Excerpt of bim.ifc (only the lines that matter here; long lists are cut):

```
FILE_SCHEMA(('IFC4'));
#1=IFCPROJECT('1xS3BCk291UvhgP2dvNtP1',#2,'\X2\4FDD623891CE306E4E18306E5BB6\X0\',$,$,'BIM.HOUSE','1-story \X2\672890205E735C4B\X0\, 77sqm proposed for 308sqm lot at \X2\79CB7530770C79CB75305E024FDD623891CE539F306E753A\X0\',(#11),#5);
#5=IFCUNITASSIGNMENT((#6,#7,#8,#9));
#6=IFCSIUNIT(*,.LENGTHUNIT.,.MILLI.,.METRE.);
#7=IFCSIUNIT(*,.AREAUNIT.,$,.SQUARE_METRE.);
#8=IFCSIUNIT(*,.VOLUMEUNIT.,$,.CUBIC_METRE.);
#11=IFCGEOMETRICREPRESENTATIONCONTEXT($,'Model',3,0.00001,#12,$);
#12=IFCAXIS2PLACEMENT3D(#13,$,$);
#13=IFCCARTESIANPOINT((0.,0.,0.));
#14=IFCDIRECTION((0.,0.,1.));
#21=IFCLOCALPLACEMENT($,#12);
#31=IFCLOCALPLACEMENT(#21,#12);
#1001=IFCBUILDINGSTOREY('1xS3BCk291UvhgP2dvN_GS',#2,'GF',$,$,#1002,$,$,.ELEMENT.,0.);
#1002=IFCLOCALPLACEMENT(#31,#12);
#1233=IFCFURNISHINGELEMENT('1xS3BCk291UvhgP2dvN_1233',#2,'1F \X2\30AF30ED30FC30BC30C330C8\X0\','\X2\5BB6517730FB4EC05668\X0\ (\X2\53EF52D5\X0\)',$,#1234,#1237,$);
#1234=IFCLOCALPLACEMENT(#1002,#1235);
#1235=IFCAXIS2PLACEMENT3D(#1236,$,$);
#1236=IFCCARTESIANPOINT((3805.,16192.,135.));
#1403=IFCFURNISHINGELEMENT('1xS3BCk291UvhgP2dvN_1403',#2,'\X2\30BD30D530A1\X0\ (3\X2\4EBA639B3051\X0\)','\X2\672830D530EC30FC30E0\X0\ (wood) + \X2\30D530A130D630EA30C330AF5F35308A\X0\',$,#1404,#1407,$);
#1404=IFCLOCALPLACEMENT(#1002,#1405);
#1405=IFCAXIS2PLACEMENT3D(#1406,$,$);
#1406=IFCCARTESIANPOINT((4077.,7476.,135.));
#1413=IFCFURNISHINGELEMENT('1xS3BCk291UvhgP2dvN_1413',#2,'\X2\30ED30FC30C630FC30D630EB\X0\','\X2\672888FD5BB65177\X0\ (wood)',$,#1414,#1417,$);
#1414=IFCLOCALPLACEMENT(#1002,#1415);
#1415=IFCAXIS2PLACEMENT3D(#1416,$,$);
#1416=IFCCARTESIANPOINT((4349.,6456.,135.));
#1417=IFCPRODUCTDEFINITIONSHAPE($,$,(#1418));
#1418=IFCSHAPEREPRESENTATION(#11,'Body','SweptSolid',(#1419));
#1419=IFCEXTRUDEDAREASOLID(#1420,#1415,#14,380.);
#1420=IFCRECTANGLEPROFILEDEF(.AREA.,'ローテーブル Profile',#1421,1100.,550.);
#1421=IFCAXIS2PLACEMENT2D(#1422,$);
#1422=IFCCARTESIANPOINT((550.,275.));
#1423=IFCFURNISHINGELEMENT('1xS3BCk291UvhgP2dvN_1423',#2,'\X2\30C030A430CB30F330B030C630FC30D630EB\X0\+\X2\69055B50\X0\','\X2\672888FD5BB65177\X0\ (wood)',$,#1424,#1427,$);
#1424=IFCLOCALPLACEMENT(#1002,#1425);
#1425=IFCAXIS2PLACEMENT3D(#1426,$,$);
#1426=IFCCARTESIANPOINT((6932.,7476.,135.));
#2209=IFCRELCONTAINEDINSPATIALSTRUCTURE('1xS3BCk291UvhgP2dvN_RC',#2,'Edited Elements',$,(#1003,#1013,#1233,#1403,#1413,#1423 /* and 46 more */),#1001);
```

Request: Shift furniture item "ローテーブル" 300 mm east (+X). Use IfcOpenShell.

```python
import ifcopenshell
import ifcopenshell.api.geometry
import ifcopenshell.util.placement

model = ifcopenshell.open("bim.ifc")

item = model.by_id(1413)
matrix = ifcopenshell.util.placement.get_local_placement(item.ObjectPlacement)
matrix[0, 3] += 300.0
ifcopenshell.api.geometry.edit_object_placement(model, product=item, matrix=matrix, is_si=False)

print(ifcopenshell.util.placement.get_local_placement(item.ObjectPlacement).round(3) + 0.0)

model.write("bim-out.ifc")
```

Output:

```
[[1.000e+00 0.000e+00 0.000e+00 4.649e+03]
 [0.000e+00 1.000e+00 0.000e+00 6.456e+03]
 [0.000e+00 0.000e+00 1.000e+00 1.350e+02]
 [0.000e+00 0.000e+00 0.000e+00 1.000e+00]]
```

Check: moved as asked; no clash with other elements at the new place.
